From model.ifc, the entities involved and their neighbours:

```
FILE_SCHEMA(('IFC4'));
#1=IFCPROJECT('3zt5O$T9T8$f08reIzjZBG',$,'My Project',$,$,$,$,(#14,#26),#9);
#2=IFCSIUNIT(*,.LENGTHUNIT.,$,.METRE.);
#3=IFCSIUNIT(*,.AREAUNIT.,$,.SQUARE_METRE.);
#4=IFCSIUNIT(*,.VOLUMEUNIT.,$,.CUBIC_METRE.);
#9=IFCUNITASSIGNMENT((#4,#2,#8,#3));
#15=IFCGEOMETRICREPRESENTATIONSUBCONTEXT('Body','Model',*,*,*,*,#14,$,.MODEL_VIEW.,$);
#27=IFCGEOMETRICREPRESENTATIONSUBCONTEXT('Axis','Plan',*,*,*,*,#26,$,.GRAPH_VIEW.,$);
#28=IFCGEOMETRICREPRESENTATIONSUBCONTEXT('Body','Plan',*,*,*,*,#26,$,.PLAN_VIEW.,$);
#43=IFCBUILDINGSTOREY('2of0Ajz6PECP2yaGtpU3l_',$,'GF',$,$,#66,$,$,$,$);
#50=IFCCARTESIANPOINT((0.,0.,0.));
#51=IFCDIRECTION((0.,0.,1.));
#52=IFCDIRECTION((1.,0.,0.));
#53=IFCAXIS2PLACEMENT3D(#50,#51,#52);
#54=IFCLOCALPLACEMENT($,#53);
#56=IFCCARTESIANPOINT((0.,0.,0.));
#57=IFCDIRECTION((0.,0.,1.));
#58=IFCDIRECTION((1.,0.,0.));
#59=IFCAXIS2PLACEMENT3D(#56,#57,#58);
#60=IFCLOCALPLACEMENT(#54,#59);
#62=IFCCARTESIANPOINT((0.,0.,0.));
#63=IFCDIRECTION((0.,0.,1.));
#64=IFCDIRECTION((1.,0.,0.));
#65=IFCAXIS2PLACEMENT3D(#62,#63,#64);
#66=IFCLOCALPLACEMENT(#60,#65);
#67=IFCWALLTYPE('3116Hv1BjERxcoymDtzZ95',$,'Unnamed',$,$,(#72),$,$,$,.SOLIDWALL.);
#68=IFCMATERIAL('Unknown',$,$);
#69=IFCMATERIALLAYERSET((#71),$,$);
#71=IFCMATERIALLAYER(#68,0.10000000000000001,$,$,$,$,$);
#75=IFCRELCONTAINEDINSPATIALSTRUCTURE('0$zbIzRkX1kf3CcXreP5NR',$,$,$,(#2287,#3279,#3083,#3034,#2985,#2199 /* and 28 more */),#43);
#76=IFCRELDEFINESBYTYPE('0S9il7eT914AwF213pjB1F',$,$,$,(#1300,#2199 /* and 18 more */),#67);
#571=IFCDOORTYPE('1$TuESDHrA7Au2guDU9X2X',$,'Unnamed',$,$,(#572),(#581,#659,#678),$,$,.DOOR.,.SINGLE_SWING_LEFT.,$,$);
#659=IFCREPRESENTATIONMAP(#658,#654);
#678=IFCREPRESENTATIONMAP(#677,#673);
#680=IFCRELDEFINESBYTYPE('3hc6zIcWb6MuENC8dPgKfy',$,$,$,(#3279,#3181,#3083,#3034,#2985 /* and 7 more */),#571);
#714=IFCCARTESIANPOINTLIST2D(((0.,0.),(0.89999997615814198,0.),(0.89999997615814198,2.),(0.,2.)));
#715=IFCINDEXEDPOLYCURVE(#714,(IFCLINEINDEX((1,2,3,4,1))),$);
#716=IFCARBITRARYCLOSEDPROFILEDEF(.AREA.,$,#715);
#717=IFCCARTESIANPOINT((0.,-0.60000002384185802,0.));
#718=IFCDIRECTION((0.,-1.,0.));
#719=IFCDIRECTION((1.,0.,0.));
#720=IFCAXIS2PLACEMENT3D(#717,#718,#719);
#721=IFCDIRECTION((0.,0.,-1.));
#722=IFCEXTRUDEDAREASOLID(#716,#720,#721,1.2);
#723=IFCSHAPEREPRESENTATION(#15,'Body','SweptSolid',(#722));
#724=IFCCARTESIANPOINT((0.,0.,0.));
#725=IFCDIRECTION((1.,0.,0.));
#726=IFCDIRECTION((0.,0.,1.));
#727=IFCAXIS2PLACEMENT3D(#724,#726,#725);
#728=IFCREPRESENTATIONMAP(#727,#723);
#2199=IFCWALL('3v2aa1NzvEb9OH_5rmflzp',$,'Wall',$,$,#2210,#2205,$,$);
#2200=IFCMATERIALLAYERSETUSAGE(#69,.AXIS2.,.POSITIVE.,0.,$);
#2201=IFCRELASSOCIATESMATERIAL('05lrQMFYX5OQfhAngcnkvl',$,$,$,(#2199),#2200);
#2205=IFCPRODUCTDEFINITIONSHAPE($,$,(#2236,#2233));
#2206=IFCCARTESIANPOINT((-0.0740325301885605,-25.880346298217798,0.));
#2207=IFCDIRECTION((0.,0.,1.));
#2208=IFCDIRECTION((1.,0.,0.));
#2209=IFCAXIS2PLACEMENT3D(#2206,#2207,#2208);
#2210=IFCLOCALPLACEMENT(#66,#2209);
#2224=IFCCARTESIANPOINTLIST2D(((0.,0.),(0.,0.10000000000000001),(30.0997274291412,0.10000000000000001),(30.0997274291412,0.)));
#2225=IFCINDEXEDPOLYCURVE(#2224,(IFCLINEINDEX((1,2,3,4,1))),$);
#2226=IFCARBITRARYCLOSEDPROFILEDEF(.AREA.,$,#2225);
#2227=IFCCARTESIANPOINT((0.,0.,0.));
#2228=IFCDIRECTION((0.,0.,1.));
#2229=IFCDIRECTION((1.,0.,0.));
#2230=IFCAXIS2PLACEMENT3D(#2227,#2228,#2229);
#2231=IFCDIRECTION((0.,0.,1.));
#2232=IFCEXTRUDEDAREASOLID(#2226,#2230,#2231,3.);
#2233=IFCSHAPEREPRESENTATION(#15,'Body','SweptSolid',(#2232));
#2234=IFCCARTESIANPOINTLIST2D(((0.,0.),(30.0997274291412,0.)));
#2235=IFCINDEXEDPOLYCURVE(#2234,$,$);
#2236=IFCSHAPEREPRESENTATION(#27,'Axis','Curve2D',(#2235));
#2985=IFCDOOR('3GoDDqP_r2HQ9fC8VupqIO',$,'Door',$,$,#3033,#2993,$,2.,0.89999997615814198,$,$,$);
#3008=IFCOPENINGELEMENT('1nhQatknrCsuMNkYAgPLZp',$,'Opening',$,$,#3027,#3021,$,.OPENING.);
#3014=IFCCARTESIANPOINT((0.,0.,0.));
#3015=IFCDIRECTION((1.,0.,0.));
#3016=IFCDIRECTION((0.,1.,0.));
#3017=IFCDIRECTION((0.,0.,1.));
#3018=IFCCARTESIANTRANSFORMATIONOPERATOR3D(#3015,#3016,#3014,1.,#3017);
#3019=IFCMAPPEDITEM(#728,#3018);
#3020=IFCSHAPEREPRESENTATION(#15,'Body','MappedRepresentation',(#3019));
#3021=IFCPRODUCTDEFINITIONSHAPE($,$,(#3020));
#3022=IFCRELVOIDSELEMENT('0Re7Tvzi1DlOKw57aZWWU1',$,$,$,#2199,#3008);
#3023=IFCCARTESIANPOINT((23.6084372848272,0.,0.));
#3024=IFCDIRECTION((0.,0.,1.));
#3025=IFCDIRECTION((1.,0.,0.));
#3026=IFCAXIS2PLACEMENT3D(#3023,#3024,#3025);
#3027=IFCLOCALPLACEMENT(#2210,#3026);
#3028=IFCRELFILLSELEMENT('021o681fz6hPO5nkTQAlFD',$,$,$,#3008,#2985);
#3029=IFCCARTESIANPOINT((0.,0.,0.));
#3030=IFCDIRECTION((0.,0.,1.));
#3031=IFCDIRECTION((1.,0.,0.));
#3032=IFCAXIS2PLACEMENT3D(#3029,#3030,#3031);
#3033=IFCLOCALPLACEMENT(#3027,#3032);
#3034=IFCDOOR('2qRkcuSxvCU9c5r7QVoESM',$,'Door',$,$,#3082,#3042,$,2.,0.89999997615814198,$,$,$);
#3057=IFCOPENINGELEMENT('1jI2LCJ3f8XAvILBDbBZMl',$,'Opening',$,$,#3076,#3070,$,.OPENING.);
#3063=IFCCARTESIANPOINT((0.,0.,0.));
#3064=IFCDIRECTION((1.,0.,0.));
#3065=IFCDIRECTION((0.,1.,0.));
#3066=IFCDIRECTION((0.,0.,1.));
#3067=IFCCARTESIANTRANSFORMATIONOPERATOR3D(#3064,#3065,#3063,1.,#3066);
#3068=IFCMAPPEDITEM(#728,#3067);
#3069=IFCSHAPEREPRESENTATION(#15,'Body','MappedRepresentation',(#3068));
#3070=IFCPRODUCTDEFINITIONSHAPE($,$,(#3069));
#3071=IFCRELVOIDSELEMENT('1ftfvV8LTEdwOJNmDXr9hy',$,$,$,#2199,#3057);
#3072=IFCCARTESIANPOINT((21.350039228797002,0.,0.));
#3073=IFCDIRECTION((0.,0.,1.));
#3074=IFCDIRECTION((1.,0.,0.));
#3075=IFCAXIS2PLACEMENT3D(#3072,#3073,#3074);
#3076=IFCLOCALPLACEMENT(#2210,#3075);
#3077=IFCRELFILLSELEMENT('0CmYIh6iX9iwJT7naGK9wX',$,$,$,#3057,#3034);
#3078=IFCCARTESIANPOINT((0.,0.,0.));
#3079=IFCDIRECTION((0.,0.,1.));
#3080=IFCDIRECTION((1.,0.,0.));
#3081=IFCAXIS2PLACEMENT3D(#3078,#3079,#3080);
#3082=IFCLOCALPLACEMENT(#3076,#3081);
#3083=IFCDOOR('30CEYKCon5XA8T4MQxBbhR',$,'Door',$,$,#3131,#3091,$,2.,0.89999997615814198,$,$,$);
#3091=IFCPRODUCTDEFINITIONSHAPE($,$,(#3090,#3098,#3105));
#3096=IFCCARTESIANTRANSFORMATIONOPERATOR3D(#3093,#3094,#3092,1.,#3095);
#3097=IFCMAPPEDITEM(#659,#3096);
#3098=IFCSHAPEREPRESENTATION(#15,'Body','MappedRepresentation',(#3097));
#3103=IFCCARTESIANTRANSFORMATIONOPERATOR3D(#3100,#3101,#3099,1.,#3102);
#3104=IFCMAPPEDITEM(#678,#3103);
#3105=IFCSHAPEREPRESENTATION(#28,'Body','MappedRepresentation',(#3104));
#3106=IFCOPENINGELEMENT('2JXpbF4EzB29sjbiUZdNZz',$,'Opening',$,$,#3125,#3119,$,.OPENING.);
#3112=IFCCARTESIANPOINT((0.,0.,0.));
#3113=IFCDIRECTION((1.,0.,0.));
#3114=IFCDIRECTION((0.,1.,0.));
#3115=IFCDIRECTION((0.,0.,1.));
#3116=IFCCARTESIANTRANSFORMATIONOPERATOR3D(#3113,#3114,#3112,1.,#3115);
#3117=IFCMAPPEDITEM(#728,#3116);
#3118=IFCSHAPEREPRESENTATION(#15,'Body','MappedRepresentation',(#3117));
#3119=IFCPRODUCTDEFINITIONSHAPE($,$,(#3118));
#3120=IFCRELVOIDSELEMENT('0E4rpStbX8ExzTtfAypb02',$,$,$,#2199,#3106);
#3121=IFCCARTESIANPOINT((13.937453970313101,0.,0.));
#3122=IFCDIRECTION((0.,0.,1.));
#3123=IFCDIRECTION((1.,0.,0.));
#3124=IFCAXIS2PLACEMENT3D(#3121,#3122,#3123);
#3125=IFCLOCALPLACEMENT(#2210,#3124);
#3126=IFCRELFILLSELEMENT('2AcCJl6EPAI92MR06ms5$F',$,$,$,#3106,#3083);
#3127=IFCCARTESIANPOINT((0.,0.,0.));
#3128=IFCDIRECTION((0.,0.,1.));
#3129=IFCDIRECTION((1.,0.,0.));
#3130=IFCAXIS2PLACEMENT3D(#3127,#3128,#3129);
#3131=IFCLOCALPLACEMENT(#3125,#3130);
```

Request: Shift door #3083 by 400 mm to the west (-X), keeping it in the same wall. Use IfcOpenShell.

```python
import ifcopenshell
import ifcopenshell.api.geometry
import ifcopenshell.util.placement
import ifcopenshell.util.unit

model = ifcopenshell.open("model.ifc")
unit_scale = ifcopenshell.util.unit.calculate_unit_scale(model)

door = model.by_guid("30CEYKCon5XA8T4MQxBbhR")
opening = door.FillsVoids[0].RelatingOpeningElement
wall = opening.VoidsElements[0].RelatingBuildingElement

wall_matrix = ifcopenshell.util.placement.get_local_placement(wall.ObjectPlacement)
shift = wall_matrix[:3, 0] * -0.4 / unit_scale
before = ifcopenshell.util.placement.get_local_placement(door.ObjectPlacement)[:3, 3].copy()

# The door is placed relative to its opening, so it follows when the opening moves.
matrix = ifcopenshell.util.placement.get_local_placement(opening.ObjectPlacement)
matrix[:3, 3] += shift
ifcopenshell.api.geometry.edit_object_placement(
    model, product=opening, matrix=matrix, is_si=False, should_transform_children=True
)

after = ifcopenshell.util.placement.get_local_placement(door.ObjectPlacement)[:3, 3]
print("door moved by", (after - before).round(3) + 0.0)

model.write("model_v2.ifc")
```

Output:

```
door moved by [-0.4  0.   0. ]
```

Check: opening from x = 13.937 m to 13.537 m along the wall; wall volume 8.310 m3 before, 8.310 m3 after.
